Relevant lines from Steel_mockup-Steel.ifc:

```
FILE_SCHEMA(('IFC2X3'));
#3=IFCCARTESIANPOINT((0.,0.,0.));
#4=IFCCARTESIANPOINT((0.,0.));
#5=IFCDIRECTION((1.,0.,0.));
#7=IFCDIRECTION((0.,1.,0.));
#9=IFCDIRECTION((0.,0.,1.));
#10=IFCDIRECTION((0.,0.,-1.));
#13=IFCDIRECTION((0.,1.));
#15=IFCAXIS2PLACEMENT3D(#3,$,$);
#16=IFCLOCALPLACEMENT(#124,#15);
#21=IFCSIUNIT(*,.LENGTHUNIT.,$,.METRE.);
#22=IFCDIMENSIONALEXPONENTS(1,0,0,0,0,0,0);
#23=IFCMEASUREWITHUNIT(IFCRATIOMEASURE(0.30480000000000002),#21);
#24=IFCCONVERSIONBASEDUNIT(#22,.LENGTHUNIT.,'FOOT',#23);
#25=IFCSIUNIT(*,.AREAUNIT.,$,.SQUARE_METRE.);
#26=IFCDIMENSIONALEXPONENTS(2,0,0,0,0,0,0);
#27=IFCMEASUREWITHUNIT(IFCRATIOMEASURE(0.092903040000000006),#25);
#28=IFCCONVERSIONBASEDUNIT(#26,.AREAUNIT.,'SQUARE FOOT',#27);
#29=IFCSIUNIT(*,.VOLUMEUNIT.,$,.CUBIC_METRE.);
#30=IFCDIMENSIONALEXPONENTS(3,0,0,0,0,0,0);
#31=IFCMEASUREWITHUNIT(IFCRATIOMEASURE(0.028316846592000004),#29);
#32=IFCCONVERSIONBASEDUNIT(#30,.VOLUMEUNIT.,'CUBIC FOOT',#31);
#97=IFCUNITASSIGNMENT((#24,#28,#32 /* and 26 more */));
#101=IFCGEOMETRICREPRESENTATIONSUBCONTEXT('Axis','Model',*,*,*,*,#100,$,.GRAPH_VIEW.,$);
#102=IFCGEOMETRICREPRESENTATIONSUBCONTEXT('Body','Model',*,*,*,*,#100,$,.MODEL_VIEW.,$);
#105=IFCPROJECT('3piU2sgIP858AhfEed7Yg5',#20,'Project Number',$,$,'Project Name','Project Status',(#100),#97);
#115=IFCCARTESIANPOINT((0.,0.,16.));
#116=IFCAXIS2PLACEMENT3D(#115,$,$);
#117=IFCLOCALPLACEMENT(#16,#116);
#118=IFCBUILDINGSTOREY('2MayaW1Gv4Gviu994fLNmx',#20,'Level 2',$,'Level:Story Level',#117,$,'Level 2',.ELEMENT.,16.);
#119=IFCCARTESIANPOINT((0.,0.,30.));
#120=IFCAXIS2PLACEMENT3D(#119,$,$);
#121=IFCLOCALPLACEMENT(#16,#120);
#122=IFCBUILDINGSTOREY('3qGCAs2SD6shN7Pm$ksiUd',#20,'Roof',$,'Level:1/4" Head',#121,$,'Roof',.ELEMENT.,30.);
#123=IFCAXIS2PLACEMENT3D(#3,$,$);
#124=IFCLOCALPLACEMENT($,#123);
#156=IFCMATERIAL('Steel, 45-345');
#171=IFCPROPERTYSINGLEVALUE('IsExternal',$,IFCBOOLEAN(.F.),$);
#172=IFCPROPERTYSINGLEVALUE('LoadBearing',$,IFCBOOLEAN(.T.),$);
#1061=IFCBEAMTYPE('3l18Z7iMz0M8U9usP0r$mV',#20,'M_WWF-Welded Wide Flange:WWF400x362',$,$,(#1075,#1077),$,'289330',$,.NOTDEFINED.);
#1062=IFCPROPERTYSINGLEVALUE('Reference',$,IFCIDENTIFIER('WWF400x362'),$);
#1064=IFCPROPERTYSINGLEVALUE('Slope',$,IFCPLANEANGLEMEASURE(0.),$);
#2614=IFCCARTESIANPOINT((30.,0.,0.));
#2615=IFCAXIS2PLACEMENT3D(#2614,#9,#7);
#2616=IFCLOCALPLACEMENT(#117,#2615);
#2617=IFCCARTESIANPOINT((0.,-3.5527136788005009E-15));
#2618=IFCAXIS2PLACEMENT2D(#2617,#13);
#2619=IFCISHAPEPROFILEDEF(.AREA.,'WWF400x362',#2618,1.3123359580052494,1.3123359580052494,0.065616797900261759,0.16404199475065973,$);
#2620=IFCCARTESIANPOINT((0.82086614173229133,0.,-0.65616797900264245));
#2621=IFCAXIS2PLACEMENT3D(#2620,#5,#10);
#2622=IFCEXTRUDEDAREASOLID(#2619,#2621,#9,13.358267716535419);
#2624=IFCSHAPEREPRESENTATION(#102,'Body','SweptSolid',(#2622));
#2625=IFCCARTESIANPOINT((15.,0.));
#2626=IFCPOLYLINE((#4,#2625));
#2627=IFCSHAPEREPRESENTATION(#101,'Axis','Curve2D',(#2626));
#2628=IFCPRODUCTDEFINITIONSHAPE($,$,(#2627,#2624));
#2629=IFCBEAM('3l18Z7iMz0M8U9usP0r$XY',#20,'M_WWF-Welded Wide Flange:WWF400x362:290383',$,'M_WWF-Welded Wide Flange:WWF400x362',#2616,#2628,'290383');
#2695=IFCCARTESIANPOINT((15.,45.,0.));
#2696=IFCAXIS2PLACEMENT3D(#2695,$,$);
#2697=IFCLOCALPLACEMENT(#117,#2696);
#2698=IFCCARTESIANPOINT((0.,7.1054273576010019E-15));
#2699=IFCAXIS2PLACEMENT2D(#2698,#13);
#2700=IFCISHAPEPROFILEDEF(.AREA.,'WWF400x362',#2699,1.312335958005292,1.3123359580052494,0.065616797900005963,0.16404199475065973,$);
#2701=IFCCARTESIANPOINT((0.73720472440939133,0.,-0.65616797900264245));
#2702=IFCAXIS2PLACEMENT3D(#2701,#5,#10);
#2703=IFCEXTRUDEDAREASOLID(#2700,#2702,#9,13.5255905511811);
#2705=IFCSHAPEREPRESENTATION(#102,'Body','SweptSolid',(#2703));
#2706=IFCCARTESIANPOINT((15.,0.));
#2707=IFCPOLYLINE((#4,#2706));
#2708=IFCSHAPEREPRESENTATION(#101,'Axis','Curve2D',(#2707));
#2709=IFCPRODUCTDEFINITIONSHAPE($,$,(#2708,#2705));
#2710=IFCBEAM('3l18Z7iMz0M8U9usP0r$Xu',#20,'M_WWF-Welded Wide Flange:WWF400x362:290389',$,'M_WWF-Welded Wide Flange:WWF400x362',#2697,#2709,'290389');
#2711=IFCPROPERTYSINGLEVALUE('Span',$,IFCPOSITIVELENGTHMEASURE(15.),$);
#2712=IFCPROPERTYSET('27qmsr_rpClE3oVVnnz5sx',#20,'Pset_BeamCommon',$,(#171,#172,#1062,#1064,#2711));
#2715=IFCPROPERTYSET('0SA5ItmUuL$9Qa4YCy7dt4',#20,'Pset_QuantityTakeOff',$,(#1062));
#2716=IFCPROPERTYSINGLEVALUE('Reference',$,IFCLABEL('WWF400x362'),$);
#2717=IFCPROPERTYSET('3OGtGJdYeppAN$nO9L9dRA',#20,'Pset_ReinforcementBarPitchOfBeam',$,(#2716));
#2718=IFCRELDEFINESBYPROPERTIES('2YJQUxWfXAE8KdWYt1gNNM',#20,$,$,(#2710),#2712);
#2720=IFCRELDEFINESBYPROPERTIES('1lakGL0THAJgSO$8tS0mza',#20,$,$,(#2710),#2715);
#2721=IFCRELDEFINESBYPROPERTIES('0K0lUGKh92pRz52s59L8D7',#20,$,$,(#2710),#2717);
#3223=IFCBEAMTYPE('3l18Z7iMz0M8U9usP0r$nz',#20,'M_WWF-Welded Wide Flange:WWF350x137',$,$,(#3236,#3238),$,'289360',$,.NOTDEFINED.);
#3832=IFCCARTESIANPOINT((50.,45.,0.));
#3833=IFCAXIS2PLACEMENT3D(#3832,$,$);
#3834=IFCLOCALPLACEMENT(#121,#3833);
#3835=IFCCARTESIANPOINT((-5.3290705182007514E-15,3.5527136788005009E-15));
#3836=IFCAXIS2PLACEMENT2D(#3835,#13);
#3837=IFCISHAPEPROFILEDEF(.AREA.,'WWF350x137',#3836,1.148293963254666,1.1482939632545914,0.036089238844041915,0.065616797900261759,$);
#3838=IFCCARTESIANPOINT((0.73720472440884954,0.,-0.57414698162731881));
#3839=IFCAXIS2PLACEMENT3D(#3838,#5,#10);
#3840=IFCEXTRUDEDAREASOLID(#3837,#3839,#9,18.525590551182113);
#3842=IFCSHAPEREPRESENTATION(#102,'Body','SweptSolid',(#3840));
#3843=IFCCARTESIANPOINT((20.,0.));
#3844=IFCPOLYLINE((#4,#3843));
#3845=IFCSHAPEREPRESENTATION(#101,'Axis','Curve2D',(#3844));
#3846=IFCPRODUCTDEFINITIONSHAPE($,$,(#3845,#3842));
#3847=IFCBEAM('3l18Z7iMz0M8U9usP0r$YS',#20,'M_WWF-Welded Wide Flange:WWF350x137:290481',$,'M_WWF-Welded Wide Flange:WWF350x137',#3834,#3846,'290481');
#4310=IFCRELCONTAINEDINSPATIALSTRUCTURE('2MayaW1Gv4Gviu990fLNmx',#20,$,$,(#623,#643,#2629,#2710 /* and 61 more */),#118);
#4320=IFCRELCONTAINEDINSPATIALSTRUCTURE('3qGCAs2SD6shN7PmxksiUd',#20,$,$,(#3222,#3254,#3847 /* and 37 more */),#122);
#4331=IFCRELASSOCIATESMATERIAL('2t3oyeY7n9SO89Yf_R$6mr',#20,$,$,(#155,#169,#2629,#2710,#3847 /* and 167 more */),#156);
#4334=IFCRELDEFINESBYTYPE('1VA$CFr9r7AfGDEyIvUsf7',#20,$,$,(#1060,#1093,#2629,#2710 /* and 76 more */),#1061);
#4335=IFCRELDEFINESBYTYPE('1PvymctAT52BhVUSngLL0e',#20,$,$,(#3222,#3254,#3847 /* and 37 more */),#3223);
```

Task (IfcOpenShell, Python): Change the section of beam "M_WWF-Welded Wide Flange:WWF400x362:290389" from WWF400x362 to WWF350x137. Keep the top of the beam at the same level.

```python
import ifcopenshell
import ifcopenshell.api.pset
import ifcopenshell.api.type
import ifcopenshell.util.element
import ifcopenshell.util.representation

model = ifcopenshell.open("Steel_mockup-Steel.ifc")

member = model.by_guid("3l18Z7iMz0M8U9usP0r$Xu")
source = next(p for p in model.by_type("IfcIShapeProfileDef") if p.ProfileName == "WWF350x137")

body = ifcopenshell.util.representation.get_representation(member, "Model", "Body")
solid = body.Items[0]
old_profile = solid.SweptArea

# Copy the section's sizes but keep this member's own profile position.
profile = ifcopenshell.util.element.copy(model, source)
# Profiles are centred, so shift by half the change in depth to hold the top.
shift = (old_profile.OverallDepth - profile.OverallDepth) / 2
x, y = old_profile.Position.Location.Coordinates
up = (-1.0, 0.0)  # upwards, in the solid's own plane
location = model.createIfcCartesianPoint((x + up[0] * shift, y + up[1] * shift))
profile.Position = model.createIfcAxis2Placement2D(location, old_profile.Position.RefDirection)
solid.SweptArea = profile
if not model.get_total_inverses(old_profile):
    ifcopenshell.util.element.remove_deep2(model, old_profile)

new_type = model.by_guid("3l18Z7iMz0M8U9usP0r$nz")
ifcopenshell.api.type.assign_type(
    model, related_objects=[member], relating_type=new_type, should_map_representations=False
)
member.Name = member.Name.replace("WWF400x362", "WWF350x137")
member.ObjectType = "M_WWF-Welded Wide Flange:WWF350x137"
pset = model.by_id(ifcopenshell.util.element.get_pset(member, "Pset_BeamCommon", should_inherit=False)["id"])
ifcopenshell.api.pset.edit_pset(model, pset=pset, properties={"Reference": "WWF350x137"})
pset = model.by_id(ifcopenshell.util.element.get_pset(member, "Pset_QuantityTakeOff", should_inherit=False)["id"])
ifcopenshell.api.pset.edit_pset(model, pset=pset, properties={"Reference": "WWF350x137"})
pset = model.by_id(ifcopenshell.util.element.get_pset(member, "Pset_ReinforcementBarPitchOfBeam", should_inherit=False)["id"])
ifcopenshell.api.pset.edit_pset(model, pset=pset, properties={"Reference": "WWF350x137"})

print(solid.SweptArea)

model.write("Steel_mockup-Steel_v2.ifc")
```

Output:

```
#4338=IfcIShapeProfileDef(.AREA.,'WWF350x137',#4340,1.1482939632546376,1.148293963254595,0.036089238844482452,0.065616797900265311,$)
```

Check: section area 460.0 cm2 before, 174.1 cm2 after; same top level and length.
